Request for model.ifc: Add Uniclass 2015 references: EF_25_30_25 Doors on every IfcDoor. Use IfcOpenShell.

First a look at what the model holds.

```python
import ifcopenshell

model = ifcopenshell.open("model.ifc")
print(model.schema)
print("classifications:", [c.Name for c in model.by_type("IfcClassification")])
for ifc_class in ("IfcDoor", "IfcRoof", "IfcStair", "IfcWall", "IfcWindow"):
    print(ifc_class, len(model.by_type(ifc_class)))
```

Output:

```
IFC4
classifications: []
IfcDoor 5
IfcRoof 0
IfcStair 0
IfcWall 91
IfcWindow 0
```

```python
import ifcopenshell
import ifcopenshell.api.classification

model = ifcopenshell.open("model.ifc")

system = ifcopenshell.api.classification.add_classification(model, classification="Uniclass 2015")

codes = {
    "IfcDoor": ("EF_25_30_25", "Doors"),
}
for ifc_class, (code, name) in codes.items():
    products = model.by_type(ifc_class)
    ifcopenshell.api.classification.add_reference(
        model, products=products, classification=system, identification=code, name=name
    )
    print(code, len(products))

model.write("model_rev.ifc")
```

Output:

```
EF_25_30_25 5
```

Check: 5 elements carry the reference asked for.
